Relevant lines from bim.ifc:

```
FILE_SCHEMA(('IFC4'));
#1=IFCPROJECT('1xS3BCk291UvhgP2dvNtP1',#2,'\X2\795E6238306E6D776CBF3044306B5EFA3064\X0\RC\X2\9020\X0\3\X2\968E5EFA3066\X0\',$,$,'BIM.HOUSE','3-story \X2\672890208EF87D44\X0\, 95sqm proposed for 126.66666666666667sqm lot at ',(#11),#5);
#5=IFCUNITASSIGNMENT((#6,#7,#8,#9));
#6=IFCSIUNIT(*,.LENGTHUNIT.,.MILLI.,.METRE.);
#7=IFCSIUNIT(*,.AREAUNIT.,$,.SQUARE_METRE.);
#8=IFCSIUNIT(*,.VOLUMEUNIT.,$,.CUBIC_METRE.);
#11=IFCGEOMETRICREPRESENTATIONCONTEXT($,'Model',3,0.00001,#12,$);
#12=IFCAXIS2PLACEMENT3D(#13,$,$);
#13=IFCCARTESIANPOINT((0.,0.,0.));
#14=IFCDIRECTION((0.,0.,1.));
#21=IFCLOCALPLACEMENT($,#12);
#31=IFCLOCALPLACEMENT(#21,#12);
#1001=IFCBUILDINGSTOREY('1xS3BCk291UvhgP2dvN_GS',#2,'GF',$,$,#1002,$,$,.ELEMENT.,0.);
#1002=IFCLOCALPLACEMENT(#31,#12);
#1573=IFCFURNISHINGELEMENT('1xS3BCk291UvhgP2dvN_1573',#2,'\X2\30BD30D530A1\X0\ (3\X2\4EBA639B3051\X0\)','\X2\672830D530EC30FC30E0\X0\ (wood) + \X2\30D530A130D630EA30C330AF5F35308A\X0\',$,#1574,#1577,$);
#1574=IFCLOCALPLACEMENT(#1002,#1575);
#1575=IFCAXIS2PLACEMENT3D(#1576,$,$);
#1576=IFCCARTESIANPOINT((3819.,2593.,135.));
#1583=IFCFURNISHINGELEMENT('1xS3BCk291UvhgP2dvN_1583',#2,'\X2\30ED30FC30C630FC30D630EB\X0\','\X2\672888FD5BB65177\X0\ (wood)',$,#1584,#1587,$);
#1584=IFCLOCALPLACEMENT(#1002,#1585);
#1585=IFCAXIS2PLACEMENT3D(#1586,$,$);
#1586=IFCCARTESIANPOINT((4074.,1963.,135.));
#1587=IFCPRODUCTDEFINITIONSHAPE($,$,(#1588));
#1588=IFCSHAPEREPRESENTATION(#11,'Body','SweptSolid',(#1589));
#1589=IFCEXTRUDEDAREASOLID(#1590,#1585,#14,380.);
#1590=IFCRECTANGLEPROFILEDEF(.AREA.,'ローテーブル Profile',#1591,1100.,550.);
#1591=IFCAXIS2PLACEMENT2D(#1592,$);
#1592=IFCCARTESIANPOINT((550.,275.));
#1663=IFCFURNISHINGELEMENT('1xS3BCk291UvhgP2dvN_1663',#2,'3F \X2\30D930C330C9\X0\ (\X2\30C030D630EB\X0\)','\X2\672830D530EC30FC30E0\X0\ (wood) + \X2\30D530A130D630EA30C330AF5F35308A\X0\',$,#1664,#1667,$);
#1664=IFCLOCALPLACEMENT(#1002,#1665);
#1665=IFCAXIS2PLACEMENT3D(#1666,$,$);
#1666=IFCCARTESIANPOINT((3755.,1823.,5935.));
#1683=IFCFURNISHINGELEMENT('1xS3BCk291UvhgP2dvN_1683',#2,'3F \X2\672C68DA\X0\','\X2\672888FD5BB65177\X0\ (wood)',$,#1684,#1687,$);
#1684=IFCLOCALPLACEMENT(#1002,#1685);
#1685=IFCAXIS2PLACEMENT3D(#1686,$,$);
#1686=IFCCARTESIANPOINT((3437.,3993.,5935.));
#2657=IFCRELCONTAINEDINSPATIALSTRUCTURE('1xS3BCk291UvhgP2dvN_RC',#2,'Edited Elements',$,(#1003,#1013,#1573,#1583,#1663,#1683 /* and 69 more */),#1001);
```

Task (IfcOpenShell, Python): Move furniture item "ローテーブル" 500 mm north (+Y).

```python
import ifcopenshell
import ifcopenshell.api.geometry
import ifcopenshell.util.placement
import ifcopenshell.util.unit

model = ifcopenshell.open("bim.ifc")
unit_scale = ifcopenshell.util.unit.calculate_unit_scale(model)

item = model.by_guid("1xS3BCk291UvhgP2dvN_1583")
matrix = ifcopenshell.util.placement.get_local_placement(item.ObjectPlacement)
matrix[1, 3] += 0.5 / unit_scale
ifcopenshell.api.geometry.edit_object_placement(model, product=item, matrix=matrix, is_si=False)

print(ifcopenshell.util.placement.get_local_placement(item.ObjectPlacement).round(3) + 0.0)

model.write("bim_edited.ifc")
```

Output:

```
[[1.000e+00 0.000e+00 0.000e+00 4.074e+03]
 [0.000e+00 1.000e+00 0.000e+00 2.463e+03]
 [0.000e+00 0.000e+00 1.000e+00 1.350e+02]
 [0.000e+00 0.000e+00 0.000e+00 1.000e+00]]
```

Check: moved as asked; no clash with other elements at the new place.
